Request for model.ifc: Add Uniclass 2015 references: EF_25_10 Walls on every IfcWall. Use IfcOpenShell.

First a look at what the model holds.

```python
import ifcopenshell

model = ifcopenshell.open("model.ifc")
print(model.schema)
print("classifications:", [c.Name for c in model.by_type("IfcClassification")])
for ifc_class in ("IfcDoor", "IfcRoof", "IfcStair", "IfcWall", "IfcWindow"):
    print(ifc_class, len(model.by_type(ifc_class)))
```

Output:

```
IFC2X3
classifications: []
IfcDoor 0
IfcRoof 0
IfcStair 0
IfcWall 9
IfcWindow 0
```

```python
import ifcopenshell
import ifcopenshell.api.classification

model = ifcopenshell.open("model.ifc")

# IFC2X3 requires Source and Edition and has no link from the project to the system.
system = model.create_entity("IfcClassification", Source="NBS", Edition="2015", Name="Uniclass 2015")

codes = {
    "IfcWall": ("EF_25_10", "Walls"),
}
for ifc_class, (code, name) in codes.items():
    products = model.by_type(ifc_class)
    ifcopenshell.api.classification.add_reference(
        model, products=products, classification=system, identification=code, name=name
    )
    print(code, len(products))

model.write("model_rev.ifc")
```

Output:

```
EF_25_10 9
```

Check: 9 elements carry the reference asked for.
